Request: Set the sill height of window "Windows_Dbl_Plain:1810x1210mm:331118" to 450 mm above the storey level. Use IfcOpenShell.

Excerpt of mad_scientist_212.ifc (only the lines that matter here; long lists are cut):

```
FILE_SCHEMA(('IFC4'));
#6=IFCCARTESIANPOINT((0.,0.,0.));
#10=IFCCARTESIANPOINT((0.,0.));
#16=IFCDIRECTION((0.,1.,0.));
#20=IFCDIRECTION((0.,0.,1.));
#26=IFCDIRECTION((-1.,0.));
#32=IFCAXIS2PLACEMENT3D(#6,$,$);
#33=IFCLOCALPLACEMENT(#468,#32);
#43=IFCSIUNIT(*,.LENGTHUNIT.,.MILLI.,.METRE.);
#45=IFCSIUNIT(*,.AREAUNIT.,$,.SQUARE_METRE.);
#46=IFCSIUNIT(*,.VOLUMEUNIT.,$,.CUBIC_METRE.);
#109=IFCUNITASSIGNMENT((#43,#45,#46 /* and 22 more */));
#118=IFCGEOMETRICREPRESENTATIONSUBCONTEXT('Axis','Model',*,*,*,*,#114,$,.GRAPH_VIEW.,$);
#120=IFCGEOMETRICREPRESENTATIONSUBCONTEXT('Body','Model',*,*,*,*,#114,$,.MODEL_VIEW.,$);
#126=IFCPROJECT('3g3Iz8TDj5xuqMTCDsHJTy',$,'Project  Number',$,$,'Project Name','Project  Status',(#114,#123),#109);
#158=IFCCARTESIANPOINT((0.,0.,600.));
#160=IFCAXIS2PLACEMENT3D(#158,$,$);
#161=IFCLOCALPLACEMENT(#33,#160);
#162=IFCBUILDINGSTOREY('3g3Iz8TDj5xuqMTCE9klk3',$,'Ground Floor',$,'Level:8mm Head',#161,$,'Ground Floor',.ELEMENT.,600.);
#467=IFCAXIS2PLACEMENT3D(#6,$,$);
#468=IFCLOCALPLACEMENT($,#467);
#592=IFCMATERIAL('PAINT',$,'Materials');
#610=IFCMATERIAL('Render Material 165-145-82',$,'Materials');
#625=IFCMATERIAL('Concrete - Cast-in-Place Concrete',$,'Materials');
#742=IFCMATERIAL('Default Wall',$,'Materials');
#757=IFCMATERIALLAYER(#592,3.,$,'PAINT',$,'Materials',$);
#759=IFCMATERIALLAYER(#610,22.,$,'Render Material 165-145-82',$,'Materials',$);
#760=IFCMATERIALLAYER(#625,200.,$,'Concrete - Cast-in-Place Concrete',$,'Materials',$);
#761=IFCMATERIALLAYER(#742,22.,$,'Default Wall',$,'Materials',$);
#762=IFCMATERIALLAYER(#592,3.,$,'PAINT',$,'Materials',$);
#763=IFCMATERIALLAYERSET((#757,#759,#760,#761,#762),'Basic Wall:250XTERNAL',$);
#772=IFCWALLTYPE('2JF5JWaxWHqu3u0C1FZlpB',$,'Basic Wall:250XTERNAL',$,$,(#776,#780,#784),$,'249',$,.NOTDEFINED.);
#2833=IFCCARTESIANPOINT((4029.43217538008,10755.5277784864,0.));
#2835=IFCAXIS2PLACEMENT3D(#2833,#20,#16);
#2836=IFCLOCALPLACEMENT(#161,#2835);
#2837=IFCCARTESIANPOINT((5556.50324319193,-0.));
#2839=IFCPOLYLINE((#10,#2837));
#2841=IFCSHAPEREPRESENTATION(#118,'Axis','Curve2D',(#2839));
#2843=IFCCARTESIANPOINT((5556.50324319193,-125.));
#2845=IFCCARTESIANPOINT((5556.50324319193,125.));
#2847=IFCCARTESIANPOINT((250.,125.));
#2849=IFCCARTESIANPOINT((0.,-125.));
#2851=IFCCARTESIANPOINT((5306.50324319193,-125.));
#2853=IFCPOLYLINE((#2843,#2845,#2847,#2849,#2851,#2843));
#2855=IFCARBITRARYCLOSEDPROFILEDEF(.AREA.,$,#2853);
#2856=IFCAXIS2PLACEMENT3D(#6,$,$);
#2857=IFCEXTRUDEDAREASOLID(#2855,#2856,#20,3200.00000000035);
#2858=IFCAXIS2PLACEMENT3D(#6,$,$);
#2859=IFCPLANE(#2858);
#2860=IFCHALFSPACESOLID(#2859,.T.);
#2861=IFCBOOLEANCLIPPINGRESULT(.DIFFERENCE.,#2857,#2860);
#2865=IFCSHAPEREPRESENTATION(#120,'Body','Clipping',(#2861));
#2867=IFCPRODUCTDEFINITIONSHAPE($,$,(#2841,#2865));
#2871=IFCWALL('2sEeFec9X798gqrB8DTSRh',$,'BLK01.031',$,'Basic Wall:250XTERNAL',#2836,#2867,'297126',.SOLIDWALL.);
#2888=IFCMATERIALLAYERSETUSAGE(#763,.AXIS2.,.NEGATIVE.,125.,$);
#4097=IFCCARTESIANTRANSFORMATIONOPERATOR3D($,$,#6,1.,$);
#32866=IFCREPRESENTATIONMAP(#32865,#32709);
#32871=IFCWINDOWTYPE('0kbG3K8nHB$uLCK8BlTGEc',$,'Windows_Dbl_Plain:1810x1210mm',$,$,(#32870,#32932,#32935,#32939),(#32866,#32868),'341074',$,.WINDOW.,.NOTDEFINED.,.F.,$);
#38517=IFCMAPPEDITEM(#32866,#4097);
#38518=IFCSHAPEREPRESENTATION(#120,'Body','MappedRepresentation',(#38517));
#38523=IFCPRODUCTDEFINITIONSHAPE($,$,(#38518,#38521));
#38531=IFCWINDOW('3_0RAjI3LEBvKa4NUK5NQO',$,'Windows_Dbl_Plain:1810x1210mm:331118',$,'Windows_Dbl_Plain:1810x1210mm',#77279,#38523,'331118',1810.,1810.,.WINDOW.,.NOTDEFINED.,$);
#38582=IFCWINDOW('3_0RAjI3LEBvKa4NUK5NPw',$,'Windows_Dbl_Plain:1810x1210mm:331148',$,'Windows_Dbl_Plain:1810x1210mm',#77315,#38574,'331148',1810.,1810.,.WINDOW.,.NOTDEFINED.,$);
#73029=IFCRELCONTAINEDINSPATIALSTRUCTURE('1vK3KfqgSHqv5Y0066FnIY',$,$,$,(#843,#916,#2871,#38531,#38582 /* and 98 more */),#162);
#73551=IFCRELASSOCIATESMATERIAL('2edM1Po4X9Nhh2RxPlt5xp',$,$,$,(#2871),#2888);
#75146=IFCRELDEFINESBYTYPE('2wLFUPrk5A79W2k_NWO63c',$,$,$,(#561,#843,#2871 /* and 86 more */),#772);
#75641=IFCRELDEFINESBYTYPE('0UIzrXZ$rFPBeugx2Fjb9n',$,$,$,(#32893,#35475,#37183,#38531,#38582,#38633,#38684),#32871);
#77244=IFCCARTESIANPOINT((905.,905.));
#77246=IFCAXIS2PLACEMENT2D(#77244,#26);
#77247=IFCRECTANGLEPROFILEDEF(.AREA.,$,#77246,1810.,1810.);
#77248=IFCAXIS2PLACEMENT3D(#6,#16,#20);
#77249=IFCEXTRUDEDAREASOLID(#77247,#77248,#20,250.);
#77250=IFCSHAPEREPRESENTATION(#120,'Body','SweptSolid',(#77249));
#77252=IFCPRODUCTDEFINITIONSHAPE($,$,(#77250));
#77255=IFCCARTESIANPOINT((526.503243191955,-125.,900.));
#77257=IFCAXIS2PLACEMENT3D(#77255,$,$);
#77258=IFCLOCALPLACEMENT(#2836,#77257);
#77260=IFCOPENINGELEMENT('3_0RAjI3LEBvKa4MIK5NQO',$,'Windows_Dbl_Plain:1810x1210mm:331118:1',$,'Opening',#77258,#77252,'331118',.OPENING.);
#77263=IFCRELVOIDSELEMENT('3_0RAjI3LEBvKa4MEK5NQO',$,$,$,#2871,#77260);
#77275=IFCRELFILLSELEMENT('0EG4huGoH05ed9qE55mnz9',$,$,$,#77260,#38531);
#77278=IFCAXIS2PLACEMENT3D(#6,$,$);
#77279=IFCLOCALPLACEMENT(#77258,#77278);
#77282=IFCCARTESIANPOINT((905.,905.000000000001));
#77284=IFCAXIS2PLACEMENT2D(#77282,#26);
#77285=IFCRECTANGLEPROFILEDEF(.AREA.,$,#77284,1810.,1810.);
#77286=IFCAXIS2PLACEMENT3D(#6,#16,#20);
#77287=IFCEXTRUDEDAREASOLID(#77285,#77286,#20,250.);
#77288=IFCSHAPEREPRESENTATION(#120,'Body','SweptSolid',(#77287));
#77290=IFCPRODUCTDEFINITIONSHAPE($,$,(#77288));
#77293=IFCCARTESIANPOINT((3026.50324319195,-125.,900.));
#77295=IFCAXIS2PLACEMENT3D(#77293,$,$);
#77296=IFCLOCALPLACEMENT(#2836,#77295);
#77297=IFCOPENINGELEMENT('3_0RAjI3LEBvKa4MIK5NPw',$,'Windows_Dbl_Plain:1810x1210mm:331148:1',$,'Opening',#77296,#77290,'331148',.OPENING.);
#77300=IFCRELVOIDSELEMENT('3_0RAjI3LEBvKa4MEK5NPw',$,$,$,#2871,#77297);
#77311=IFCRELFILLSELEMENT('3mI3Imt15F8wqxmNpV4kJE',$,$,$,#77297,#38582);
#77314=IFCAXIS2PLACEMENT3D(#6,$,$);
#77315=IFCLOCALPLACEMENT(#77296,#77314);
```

```python
import numpy as np
import ifcopenshell
import ifcopenshell.api.geometry
import ifcopenshell.geom
import ifcopenshell.util.element
import ifcopenshell.util.placement
import ifcopenshell.util.shape
import ifcopenshell.util.unit

model = ifcopenshell.open("mad_scientist_212.ifc")
unit_scale = ifcopenshell.util.unit.calculate_unit_scale(model)

window = model.by_guid("3_0RAjI3LEBvKa4NUK5NQO")
opening = window.FillsVoids[0].RelatingOpeningElement
storey = ifcopenshell.util.element.get_container(window, ifc_class="IfcBuildingStorey")
level = ifcopenshell.util.placement.get_local_placement(storey.ObjectPlacement)[2, 3]

# The opening's origin need not be at the sill, so measure its lowest point.
shape = ifcopenshell.geom.create_shape(ifcopenshell.geom.settings(), opening)
bottom = ifcopenshell.util.shape.get_shape_bottom_elevation(shape, shape.geometry) / unit_scale
dz = level + 450.0 - bottom

shift = np.array([0.0, 0.0, dz])
# The window is placed relative to its opening, so it follows when the opening moves.
matrix = ifcopenshell.util.placement.get_local_placement(opening.ObjectPlacement)
matrix[:3, 3] += shift
ifcopenshell.api.geometry.edit_object_placement(
    model, product=opening, matrix=matrix, is_si=False, should_transform_children=True
)

print(f"moved by {dz * unit_scale:+.3f} m")

model.write("mad_scientist_212_edited.ifc")
```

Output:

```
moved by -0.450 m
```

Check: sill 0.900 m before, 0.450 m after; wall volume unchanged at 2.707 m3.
